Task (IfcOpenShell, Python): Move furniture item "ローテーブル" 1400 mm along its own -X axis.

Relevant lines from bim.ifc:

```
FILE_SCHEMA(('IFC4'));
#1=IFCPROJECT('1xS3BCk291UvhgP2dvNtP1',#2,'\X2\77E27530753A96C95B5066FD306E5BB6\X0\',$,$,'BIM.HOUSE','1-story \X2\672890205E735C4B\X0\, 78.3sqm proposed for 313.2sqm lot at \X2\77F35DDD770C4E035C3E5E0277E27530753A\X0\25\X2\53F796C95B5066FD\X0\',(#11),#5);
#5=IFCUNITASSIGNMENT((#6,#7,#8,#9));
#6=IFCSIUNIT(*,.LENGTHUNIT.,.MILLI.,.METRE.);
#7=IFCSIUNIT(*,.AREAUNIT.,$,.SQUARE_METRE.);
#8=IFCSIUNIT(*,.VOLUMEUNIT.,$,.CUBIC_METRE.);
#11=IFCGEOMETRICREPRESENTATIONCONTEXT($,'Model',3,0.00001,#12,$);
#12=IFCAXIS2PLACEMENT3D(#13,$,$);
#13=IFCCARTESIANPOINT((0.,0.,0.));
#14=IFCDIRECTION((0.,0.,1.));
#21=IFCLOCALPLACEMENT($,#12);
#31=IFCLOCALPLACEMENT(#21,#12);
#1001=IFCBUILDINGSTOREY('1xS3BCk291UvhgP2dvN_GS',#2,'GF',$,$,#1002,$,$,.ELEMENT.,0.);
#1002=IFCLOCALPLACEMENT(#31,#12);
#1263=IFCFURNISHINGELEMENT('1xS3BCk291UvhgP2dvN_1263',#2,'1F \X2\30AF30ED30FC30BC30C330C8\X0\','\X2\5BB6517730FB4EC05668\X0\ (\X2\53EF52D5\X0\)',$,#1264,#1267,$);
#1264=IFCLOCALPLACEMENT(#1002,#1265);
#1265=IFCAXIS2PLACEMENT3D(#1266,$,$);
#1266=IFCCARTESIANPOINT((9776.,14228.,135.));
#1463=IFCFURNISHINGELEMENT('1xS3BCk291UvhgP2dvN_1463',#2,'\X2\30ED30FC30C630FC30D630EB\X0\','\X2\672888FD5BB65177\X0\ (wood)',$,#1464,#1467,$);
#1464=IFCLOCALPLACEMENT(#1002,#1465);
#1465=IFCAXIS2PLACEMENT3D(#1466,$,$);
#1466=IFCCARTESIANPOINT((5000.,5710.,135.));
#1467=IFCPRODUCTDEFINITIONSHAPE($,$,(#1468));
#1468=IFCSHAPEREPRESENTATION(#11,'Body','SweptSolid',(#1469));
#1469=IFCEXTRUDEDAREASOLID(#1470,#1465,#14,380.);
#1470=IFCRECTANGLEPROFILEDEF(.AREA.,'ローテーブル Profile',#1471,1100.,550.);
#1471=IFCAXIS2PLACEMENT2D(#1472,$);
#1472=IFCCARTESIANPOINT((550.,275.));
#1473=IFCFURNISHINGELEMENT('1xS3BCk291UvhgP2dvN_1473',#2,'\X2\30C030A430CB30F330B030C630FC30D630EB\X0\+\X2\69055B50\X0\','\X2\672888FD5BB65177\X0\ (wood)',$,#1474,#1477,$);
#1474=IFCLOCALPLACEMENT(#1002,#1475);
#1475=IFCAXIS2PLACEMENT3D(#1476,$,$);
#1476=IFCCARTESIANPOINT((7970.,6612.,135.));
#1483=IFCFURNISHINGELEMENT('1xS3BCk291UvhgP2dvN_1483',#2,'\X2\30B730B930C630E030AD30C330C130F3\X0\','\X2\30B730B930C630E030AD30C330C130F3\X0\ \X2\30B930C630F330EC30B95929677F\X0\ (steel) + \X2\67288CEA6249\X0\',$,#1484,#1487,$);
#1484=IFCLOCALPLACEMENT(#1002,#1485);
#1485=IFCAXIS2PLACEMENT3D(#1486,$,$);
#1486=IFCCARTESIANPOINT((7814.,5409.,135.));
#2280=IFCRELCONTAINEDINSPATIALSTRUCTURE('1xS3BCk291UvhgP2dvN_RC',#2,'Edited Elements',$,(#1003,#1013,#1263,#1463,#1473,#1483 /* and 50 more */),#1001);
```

```python
import ifcopenshell
import ifcopenshell.api.geometry
import ifcopenshell.util.placement

model = ifcopenshell.open("bim.ifc")

item = model.by_guid("1xS3BCk291UvhgP2dvN_1463")
matrix = ifcopenshell.util.placement.get_local_placement(item.ObjectPlacement)
matrix[:3, 3] -= matrix[:3, 0] * 1400.0
ifcopenshell.api.geometry.edit_object_placement(model, product=item, matrix=matrix, is_si=False)

print(ifcopenshell.util.placement.get_local_placement(item.ObjectPlacement).round(3) + 0.0)

model.write("bim_v2.ifc")
```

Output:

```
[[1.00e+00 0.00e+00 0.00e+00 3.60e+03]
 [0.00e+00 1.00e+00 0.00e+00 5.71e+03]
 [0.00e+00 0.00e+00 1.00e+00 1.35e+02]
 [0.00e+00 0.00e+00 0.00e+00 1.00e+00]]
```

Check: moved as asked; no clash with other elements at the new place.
